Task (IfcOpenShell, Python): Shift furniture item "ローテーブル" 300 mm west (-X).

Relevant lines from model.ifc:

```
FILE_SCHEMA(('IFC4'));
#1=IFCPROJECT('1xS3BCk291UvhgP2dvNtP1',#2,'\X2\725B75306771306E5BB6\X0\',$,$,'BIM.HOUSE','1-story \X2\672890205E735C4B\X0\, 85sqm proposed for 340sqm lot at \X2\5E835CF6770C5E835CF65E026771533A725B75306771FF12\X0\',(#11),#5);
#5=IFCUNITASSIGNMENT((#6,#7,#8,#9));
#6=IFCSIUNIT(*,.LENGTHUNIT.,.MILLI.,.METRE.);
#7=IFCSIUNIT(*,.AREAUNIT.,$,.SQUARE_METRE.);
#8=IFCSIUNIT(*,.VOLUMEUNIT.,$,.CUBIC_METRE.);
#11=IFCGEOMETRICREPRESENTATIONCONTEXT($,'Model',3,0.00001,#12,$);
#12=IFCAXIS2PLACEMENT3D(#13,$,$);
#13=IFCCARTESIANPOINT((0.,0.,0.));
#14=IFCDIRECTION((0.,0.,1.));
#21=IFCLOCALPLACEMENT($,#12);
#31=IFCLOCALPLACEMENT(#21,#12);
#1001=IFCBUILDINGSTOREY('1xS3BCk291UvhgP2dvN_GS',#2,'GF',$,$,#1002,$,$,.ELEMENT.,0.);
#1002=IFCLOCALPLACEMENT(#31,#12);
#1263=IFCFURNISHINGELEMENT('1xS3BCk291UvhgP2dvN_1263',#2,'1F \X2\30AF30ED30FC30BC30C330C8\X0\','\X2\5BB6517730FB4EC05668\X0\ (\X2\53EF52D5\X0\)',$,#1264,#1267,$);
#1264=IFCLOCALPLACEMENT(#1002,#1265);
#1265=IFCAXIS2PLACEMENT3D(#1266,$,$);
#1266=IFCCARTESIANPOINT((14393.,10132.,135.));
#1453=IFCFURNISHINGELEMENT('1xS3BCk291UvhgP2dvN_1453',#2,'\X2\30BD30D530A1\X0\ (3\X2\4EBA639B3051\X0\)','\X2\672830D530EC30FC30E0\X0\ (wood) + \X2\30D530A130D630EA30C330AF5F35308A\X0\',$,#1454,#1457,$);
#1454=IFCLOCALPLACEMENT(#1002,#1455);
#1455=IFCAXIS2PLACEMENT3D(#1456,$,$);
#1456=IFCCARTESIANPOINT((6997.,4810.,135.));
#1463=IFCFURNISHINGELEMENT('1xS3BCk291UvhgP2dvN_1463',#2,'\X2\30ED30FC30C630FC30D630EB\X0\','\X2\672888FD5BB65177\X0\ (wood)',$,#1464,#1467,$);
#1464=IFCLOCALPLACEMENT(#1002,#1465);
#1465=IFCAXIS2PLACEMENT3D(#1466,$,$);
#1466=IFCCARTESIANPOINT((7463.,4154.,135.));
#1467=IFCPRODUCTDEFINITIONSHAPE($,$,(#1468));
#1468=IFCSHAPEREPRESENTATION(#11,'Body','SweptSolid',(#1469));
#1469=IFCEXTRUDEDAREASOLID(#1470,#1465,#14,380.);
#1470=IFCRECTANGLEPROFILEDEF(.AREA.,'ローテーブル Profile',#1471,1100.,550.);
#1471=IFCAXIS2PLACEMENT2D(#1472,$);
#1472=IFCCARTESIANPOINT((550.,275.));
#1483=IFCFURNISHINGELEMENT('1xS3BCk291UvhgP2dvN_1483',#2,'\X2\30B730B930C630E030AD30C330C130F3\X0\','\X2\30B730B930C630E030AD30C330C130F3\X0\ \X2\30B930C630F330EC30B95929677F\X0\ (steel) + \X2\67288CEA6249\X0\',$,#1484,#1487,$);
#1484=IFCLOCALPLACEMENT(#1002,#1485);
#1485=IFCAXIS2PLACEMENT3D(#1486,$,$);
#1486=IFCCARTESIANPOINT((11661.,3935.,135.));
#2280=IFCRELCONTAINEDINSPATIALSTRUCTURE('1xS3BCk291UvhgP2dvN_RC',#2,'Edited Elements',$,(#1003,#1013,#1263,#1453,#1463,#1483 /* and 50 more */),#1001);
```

```python
import ifcopenshell
import ifcopenshell.api.geometry
import ifcopenshell.util.placement
import ifcopenshell.util.unit

model = ifcopenshell.open("model.ifc")
unit_scale = ifcopenshell.util.unit.calculate_unit_scale(model)

item = model.by_guid("1xS3BCk291UvhgP2dvN_1463")
matrix = ifcopenshell.util.placement.get_local_placement(item.ObjectPlacement)
matrix[0, 3] -= 0.3 / unit_scale
ifcopenshell.api.geometry.edit_object_placement(model, product=item, matrix=matrix, is_si=False)

print(ifcopenshell.util.placement.get_local_placement(item.ObjectPlacement).round(3) + 0.0)

model.write("model_edited.ifc")
```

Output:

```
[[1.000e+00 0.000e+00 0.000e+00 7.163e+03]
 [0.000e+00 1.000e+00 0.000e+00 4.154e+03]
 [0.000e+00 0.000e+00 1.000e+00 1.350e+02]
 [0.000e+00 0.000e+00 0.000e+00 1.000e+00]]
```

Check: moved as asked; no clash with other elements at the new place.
